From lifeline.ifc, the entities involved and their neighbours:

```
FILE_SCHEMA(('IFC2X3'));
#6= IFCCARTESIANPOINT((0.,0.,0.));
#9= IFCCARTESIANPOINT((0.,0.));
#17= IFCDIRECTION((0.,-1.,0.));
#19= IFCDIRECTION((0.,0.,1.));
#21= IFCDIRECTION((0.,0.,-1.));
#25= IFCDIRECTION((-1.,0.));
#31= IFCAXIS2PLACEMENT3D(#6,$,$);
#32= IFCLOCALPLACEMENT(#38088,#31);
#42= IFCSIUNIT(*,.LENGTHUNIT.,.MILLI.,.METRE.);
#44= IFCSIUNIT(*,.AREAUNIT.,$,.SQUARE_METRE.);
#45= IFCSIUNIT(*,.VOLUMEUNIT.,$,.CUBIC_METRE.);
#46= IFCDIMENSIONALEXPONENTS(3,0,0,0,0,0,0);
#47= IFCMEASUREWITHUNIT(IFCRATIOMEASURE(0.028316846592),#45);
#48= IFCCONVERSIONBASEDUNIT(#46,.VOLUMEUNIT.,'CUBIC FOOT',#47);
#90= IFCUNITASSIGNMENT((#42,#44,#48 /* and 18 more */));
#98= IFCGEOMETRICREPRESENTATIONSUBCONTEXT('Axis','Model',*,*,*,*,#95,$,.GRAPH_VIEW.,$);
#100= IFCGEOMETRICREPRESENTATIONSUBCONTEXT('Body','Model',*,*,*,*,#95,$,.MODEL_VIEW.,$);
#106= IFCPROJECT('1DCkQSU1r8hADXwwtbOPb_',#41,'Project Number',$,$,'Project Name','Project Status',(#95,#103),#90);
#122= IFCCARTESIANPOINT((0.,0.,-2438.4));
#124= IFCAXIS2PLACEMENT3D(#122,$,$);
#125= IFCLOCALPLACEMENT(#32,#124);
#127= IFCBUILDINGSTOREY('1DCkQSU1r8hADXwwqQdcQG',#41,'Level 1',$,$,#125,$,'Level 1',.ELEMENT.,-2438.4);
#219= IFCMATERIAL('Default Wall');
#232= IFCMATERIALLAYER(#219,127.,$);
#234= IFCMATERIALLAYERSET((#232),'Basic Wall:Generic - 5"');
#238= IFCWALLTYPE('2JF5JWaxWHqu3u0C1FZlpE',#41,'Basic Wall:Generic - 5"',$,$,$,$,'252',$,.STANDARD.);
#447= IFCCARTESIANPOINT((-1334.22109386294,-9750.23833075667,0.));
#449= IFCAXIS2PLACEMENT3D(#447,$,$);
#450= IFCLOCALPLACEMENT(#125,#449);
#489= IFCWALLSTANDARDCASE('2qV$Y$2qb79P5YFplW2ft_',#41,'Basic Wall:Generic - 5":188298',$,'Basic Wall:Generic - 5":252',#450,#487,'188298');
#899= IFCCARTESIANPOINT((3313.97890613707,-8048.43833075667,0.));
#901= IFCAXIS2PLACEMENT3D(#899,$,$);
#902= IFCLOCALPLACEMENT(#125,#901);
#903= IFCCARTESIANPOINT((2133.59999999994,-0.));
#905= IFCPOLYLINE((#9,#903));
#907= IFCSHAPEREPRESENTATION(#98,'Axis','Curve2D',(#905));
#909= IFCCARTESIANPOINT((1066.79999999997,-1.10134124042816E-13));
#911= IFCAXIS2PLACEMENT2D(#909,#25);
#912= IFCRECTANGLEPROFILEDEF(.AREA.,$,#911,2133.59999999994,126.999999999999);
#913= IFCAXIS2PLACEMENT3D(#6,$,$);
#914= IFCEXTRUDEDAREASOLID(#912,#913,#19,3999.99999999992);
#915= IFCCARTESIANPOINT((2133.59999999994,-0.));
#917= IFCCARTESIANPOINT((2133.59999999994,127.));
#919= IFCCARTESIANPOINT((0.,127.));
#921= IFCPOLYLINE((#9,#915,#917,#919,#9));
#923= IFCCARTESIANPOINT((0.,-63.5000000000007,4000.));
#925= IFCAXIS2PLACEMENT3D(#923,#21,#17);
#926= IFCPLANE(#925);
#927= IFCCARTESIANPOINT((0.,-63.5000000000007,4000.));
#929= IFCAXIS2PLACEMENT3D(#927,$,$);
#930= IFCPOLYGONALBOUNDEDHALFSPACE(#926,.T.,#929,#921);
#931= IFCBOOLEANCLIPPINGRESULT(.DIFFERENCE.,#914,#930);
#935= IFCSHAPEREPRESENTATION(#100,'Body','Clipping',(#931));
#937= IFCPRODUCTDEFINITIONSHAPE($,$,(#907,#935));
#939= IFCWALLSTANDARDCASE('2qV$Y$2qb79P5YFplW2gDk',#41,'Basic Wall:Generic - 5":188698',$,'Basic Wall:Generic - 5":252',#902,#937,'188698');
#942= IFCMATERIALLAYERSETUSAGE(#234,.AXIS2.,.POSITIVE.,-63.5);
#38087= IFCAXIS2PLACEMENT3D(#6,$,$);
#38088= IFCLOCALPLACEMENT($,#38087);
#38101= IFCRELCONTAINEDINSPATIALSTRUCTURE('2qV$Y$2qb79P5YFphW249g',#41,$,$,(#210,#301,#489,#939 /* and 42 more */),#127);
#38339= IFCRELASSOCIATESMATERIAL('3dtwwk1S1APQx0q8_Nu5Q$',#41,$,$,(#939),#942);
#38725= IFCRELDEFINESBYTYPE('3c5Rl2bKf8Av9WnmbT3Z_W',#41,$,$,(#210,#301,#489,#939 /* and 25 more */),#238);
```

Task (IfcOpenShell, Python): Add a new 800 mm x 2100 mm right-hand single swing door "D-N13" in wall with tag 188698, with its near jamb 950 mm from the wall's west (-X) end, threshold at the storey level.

```python
import numpy as np
import ifcopenshell
import ifcopenshell.api.feature
import ifcopenshell.api.geometry
import ifcopenshell.api.root
import ifcopenshell.api.spatial
import ifcopenshell.api.type
import ifcopenshell.geom
import ifcopenshell.util.element
import ifcopenshell.util.placement
import ifcopenshell.util.representation
import ifcopenshell.util.shape
import ifcopenshell.util.unit

model = ifcopenshell.open("lifeline.ifc")
unit_scale = ifcopenshell.util.unit.calculate_unit_scale(model)
settings = ifcopenshell.geom.settings()


def volume(element):
    """Net volume in cubic metres, openings subtracted."""
    shape = ifcopenshell.geom.create_shape(settings, element)
    return ifcopenshell.util.shape.get_volume(shape.geometry)


wall = model.by_guid("2qV$Y$2qb79P5YFplW2gDk")
storey = ifcopenshell.util.element.get_container(wall, ifc_class="IfcBuildingStorey")
context = ifcopenshell.util.representation.get_context(model, "Model", "Body", "MODEL_VIEW")
before = volume(wall)

width, height, from_end, sill = 0.8, 2.1, 0.95, 0.0  # metres

# The wall runs along its own X axis, and the end named is its -X end.
wall_shape = ifcopenshell.geom.create_shape(settings, wall)
x, y, z = ifcopenshell.util.shape.get_vertices(wall_shape.geometry).T
start = x.min() + from_end
face, thickness = float(y.min()), float(y.max() - y.min())
wall_matrix = ifcopenshell.util.placement.get_local_placement(wall.ObjectPlacement)
level = ifcopenshell.util.placement.get_local_placement(storey.ObjectPlacement)[2, 3]


def in_wall(x, y):
    """Placement at x, y metres in the wall's axes, at sill height."""
    matrix = wall_matrix.copy()
    matrix[:, 3] = wall_matrix @ np.array([x / unit_scale, y / unit_scale, 0.0, 1.0])
    matrix[2, 3] = level + sill / unit_scale
    return matrix


# Opening: a box that overshoots both wall faces by 50 mm.
opening = ifcopenshell.api.root.create_entity(model, ifc_class="IfcOpeningElement")
box = ifcopenshell.api.geometry.add_wall_representation(
    model, context=context, length=width, height=height, thickness=thickness + 0.1
)
ifcopenshell.api.geometry.assign_representation(model, product=opening, representation=box)
ifcopenshell.api.geometry.edit_object_placement(model, product=opening, matrix=in_wall(start, face - 0.05), is_si=False)
ifcopenshell.api.feature.add_feature(model, feature=opening, element=wall)

door = ifcopenshell.api.root.create_entity(model, ifc_class="IfcDoor", name="D-N13")
door.OverallWidth, door.OverallHeight = width / unit_scale, height / unit_scale
body = ifcopenshell.api.geometry.add_door_representation(
    model,
    context=context,
    overall_width=door.OverallWidth,
    overall_height=door.OverallHeight,
    operation_type="SINGLE_SWING_RIGHT",
    lining_properties={"LiningDepth": thickness / unit_scale, "ThresholdDepth": thickness / unit_scale},
)
ifcopenshell.api.geometry.assign_representation(model, product=door, representation=body)
ifcopenshell.api.spatial.assign_container(model, products=[door], relating_structure=storey)
fills = ifcopenshell.api.feature.add_filling(model, opening=opening, element=door)
fills.OwnerHistory = door.OwnerHistory  # required in IFC2X3

# IFC2X3 keeps the operation on the door style.
style = ifcopenshell.api.root.create_entity(model, ifc_class="IfcDoorStyle", name="D-N13")
style.OperationType, style.ConstructionType = "SINGLE_SWING_RIGHT", "NOTDEFINED"
style.ParameterTakesPrecedence = style.Sizeable = False
ifcopenshell.api.type.assign_type(model, related_objects=[door], relating_type=style)

# The lining spans the wall, so the door starts at the wall face.
ifcopenshell.api.geometry.edit_object_placement(model, product=door, matrix=in_wall(start, face), is_si=False)

after = volume(wall)

print(f"wall volume {before:.3f} -> {after:.3f} m3")

model.write("lifeline_edited.ifc")
```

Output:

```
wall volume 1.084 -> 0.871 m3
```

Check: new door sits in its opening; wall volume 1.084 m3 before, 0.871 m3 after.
